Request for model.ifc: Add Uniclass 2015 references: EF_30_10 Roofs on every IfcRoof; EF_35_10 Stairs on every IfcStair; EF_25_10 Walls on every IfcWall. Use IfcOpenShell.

First a look at what the model holds.

```python
import ifcopenshell

model = ifcopenshell.open("model.ifc")
print(model.schema)
print("classifications:", [c.Name for c in model.by_type("IfcClassification")])
for ifc_class in ("IfcDoor", "IfcRoof", "IfcStair", "IfcWall", "IfcWindow"):
    print(ifc_class, len(model.by_type(ifc_class)))
```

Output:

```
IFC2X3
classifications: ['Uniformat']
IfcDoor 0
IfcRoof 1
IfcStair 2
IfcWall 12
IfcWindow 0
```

```python
import ifcopenshell
import ifcopenshell.api.classification

model = ifcopenshell.open("model.ifc")

# IFC2X3 requires Source and Edition and has no link from the project to the system.
system = model.create_entity("IfcClassification", Source="NBS", Edition="2015", Name="Uniclass 2015")

codes = {
    "IfcRoof": ("EF_30_10", "Roofs"),
    "IfcStair": ("EF_35_10", "Stairs"),
    "IfcWall": ("EF_25_10", "Walls"),
}
for ifc_class, (code, name) in codes.items():
    products = model.by_type(ifc_class)
    ifcopenshell.api.classification.add_reference(
        model, products=products, classification=system, identification=code, name=name
    )
    print(code, len(products))

model.write("model_edited.ifc")
```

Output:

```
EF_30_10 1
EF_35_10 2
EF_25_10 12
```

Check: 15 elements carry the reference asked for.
